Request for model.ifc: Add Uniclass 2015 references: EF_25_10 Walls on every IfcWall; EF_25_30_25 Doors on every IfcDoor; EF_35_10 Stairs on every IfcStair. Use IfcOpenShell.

First a look at what the model holds.

```python
import ifcopenshell

model = ifcopenshell.open("model.ifc")
print(model.schema)
print("classifications:", [c.Name for c in model.by_type("IfcClassification")])
for ifc_class in ("IfcDoor", "IfcRoof", "IfcStair", "IfcWall", "IfcWindow"):
    print(ifc_class, len(model.by_type(ifc_class)))
```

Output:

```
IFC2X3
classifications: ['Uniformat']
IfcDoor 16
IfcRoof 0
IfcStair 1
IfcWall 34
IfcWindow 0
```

```python
import ifcopenshell
import ifcopenshell.api.classification

model = ifcopenshell.open("model.ifc")

# IFC2X3 requires Source and Edition and has no link from the project to the system.
system = model.create_entity("IfcClassification", Source="NBS", Edition="2015", Name="Uniclass 2015")

codes = {
    "IfcWall": ("EF_25_10", "Walls"),
    "IfcDoor": ("EF_25_30_25", "Doors"),
    "IfcStair": ("EF_35_10", "Stairs"),
}
for ifc_class, (code, name) in codes.items():
    products = model.by_type(ifc_class)
    ifcopenshell.api.classification.add_reference(
        model, products=products, classification=system, identification=code, name=name
    )
    print(code, len(products))

model.write("model_edited.ifc")
```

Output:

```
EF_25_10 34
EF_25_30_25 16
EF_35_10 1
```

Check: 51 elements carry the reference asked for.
